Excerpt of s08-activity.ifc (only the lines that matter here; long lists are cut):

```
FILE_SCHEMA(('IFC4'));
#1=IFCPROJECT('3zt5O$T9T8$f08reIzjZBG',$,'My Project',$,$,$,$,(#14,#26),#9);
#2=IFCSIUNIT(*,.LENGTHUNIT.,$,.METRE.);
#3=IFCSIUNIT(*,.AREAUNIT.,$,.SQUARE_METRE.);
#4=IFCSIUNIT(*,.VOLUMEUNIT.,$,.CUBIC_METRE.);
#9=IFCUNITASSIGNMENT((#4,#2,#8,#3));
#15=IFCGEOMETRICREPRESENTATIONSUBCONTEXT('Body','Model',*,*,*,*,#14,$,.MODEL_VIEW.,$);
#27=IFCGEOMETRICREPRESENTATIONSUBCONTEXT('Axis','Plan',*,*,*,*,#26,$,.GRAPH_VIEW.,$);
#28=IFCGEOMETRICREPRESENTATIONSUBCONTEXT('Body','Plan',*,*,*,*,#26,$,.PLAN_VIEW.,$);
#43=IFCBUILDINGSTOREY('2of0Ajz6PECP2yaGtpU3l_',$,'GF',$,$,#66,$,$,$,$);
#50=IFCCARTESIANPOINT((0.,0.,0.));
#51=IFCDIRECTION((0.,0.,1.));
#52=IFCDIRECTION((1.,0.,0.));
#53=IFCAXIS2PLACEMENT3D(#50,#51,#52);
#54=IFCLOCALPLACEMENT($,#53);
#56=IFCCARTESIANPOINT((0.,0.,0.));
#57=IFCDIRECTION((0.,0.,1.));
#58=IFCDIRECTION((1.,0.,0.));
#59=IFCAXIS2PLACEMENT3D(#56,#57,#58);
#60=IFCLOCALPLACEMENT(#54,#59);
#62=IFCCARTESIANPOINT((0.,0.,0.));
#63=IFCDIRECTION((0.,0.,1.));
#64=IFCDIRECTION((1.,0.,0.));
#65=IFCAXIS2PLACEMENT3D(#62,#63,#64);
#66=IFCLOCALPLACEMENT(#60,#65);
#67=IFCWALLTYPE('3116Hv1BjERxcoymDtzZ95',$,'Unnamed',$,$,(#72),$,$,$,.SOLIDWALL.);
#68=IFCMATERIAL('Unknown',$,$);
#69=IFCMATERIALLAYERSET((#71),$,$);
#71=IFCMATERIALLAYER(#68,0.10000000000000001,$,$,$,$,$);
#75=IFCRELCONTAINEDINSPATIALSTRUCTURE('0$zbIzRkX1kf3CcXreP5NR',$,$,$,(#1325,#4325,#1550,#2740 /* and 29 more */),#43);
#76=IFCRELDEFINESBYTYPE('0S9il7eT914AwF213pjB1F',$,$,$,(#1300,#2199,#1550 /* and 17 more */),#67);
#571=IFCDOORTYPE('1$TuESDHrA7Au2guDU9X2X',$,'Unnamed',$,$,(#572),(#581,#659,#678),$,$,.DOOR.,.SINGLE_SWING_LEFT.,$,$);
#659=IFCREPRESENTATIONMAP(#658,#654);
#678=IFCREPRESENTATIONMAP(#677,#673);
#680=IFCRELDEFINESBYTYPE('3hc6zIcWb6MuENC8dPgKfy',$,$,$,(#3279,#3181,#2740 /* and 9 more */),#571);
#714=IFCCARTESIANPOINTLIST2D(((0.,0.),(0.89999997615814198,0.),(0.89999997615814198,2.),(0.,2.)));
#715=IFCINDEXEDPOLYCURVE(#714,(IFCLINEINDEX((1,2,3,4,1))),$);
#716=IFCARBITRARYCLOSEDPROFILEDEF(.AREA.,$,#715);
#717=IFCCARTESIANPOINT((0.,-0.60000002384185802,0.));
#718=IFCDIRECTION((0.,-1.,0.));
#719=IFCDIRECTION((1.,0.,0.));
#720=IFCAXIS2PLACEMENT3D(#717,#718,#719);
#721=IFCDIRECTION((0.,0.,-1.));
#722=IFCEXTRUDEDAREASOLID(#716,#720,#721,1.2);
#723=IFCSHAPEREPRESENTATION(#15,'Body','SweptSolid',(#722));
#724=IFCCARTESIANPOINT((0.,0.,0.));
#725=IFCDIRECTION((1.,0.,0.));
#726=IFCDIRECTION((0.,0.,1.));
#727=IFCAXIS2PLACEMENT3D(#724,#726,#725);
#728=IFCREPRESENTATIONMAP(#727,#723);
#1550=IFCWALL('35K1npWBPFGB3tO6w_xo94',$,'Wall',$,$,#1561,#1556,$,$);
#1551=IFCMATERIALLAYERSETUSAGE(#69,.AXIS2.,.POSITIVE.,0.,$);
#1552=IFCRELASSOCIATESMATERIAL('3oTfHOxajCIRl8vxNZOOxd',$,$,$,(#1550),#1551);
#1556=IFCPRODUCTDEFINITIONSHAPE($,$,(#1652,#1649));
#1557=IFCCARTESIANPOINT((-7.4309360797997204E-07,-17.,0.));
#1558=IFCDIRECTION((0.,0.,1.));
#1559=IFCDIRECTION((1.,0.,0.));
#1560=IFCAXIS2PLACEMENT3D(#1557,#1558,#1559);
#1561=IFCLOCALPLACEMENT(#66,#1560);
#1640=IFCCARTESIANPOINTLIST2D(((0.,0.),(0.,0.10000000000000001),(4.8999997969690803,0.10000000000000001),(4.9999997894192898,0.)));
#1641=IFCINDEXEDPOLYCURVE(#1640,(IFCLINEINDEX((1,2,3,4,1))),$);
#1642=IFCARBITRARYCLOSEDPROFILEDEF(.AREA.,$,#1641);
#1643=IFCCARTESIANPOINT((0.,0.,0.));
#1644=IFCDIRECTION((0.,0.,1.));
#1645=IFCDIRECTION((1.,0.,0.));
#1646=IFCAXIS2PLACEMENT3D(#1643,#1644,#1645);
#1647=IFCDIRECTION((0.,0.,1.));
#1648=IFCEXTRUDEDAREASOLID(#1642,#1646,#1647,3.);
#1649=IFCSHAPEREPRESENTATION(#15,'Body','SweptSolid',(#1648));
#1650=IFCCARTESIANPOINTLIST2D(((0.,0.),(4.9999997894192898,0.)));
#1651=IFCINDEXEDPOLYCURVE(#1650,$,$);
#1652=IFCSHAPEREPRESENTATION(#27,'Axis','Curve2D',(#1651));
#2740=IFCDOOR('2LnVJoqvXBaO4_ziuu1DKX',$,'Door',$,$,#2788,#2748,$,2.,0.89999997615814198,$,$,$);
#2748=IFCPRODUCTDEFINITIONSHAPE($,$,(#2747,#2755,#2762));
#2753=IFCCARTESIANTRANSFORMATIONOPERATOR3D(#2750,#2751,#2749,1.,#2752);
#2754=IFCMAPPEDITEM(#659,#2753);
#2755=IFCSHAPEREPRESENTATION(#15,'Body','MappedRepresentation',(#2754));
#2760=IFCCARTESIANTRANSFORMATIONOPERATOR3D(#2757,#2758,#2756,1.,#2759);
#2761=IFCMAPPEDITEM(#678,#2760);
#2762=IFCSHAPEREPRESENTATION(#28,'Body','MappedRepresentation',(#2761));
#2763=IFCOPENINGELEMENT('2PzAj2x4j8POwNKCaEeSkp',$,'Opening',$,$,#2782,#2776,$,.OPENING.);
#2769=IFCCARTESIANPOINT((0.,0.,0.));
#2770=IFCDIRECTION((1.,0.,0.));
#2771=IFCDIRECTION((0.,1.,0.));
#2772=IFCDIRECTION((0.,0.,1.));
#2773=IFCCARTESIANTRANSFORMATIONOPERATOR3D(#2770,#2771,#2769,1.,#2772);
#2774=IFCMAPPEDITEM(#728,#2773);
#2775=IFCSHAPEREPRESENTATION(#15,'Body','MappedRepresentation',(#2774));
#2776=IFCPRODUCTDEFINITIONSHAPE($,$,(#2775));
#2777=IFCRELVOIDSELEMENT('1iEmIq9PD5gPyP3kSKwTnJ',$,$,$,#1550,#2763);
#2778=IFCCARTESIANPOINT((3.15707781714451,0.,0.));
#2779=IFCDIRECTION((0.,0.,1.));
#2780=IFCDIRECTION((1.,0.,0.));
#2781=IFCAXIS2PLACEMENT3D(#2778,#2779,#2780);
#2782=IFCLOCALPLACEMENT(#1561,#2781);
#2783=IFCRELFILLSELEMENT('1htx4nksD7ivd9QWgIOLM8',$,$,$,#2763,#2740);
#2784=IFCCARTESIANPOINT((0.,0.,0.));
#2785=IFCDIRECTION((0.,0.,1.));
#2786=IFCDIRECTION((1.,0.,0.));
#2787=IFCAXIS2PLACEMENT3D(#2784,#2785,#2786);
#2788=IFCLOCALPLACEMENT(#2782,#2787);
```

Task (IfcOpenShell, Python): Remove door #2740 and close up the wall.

```python
import ifcopenshell
import ifcopenshell.api.feature
import ifcopenshell.api.root
import ifcopenshell.geom
import ifcopenshell.util.shape

model = ifcopenshell.open("s08-activity.ifc")
settings = ifcopenshell.geom.settings()


def volume(element):
    """Net volume in cubic metres, openings subtracted."""
    shape = ifcopenshell.geom.create_shape(settings, element)
    return ifcopenshell.util.shape.get_volume(shape.geometry)


door = model.by_guid("2LnVJoqvXBaO4_ziuu1DKX")
opening = door.FillsVoids[0].RelatingOpeningElement
wall = opening.VoidsElements[0].RelatingBuildingElement
before = volume(wall)

ifcopenshell.api.root.remove_product(model, product=door)
ifcopenshell.api.feature.remove_feature(model, feature=opening)

after = volume(wall)

print(f"wall volume {before:.3f} -> {after:.3f} m3")

model.write("s08-activity_updated.ifc")
```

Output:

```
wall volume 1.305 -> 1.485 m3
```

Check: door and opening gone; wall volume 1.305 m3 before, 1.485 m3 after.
